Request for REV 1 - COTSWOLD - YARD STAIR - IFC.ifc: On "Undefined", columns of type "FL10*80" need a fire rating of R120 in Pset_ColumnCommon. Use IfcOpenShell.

First a look at what the model holds.

```python
import ifcopenshell
import ifcopenshell.util.element

model = ifcopenshell.open("REV 1 - COTSWOLD - YARD STAIR - IFC.ifc")
print(model.schema)
storey = next(s for s in model.by_type("IfcBuildingStorey") if s.Name == "Undefined")
columns = [e for e in ifcopenshell.util.element.get_decomposition(storey) if e.is_a("IfcColumn")]
seen = {}
for e in columns:
    element_type = ifcopenshell.util.element.get_type(e)
    key = (element_type.Name if element_type != e and element_type else None, ifcopenshell.util.element.get_pset(e, "Pset_ColumnCommon", "FireRating"))
    seen[key] = seen.get(key, 0) + 1
for (name, value), count in sorted(seen.items(), key=str):
    print(count, "x", name, "|", value)
```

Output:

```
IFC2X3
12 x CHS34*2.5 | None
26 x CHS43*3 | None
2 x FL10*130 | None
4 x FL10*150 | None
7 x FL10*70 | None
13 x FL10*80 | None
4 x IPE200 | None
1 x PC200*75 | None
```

```python
import ifcopenshell
import ifcopenshell.api.pset
import ifcopenshell.util.element

model = ifcopenshell.open("REV 1 - COTSWOLD - YARD STAIR - IFC.ifc")

storey = next(s for s in model.by_type("IfcBuildingStorey") if s.Name == "Undefined")
columns = [e for e in ifcopenshell.util.element.get_decomposition(storey) if e.is_a("IfcColumn")]

count = 0
for e in columns:
    element_type = ifcopenshell.util.element.get_type(e)
    if element_type in (None, e) or element_type.Name != "FL10*80":
        continue
    found = ifcopenshell.util.element.get_pset(e, "Pset_ColumnCommon", should_inherit=False)
    if found:
        pset = model.by_id(found["id"])
        if len(ifcopenshell.util.element.get_elements_by_pset(pset)) > 1:
            pset = ifcopenshell.api.pset.unshare_pset(model, products=[e], pset=pset)[0]
    else:
        pset = ifcopenshell.api.pset.add_pset(model, product=e, name="Pset_ColumnCommon")
    ifcopenshell.api.pset.edit_pset(model, pset=pset, properties={"FireRating": "R120"})
    count += 1

print(count, "columns updated")

model.write("REV 1 - COTSWOLD - YARD STAIR - IFC_v2.ifc")
```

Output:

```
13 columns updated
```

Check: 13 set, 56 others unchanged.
